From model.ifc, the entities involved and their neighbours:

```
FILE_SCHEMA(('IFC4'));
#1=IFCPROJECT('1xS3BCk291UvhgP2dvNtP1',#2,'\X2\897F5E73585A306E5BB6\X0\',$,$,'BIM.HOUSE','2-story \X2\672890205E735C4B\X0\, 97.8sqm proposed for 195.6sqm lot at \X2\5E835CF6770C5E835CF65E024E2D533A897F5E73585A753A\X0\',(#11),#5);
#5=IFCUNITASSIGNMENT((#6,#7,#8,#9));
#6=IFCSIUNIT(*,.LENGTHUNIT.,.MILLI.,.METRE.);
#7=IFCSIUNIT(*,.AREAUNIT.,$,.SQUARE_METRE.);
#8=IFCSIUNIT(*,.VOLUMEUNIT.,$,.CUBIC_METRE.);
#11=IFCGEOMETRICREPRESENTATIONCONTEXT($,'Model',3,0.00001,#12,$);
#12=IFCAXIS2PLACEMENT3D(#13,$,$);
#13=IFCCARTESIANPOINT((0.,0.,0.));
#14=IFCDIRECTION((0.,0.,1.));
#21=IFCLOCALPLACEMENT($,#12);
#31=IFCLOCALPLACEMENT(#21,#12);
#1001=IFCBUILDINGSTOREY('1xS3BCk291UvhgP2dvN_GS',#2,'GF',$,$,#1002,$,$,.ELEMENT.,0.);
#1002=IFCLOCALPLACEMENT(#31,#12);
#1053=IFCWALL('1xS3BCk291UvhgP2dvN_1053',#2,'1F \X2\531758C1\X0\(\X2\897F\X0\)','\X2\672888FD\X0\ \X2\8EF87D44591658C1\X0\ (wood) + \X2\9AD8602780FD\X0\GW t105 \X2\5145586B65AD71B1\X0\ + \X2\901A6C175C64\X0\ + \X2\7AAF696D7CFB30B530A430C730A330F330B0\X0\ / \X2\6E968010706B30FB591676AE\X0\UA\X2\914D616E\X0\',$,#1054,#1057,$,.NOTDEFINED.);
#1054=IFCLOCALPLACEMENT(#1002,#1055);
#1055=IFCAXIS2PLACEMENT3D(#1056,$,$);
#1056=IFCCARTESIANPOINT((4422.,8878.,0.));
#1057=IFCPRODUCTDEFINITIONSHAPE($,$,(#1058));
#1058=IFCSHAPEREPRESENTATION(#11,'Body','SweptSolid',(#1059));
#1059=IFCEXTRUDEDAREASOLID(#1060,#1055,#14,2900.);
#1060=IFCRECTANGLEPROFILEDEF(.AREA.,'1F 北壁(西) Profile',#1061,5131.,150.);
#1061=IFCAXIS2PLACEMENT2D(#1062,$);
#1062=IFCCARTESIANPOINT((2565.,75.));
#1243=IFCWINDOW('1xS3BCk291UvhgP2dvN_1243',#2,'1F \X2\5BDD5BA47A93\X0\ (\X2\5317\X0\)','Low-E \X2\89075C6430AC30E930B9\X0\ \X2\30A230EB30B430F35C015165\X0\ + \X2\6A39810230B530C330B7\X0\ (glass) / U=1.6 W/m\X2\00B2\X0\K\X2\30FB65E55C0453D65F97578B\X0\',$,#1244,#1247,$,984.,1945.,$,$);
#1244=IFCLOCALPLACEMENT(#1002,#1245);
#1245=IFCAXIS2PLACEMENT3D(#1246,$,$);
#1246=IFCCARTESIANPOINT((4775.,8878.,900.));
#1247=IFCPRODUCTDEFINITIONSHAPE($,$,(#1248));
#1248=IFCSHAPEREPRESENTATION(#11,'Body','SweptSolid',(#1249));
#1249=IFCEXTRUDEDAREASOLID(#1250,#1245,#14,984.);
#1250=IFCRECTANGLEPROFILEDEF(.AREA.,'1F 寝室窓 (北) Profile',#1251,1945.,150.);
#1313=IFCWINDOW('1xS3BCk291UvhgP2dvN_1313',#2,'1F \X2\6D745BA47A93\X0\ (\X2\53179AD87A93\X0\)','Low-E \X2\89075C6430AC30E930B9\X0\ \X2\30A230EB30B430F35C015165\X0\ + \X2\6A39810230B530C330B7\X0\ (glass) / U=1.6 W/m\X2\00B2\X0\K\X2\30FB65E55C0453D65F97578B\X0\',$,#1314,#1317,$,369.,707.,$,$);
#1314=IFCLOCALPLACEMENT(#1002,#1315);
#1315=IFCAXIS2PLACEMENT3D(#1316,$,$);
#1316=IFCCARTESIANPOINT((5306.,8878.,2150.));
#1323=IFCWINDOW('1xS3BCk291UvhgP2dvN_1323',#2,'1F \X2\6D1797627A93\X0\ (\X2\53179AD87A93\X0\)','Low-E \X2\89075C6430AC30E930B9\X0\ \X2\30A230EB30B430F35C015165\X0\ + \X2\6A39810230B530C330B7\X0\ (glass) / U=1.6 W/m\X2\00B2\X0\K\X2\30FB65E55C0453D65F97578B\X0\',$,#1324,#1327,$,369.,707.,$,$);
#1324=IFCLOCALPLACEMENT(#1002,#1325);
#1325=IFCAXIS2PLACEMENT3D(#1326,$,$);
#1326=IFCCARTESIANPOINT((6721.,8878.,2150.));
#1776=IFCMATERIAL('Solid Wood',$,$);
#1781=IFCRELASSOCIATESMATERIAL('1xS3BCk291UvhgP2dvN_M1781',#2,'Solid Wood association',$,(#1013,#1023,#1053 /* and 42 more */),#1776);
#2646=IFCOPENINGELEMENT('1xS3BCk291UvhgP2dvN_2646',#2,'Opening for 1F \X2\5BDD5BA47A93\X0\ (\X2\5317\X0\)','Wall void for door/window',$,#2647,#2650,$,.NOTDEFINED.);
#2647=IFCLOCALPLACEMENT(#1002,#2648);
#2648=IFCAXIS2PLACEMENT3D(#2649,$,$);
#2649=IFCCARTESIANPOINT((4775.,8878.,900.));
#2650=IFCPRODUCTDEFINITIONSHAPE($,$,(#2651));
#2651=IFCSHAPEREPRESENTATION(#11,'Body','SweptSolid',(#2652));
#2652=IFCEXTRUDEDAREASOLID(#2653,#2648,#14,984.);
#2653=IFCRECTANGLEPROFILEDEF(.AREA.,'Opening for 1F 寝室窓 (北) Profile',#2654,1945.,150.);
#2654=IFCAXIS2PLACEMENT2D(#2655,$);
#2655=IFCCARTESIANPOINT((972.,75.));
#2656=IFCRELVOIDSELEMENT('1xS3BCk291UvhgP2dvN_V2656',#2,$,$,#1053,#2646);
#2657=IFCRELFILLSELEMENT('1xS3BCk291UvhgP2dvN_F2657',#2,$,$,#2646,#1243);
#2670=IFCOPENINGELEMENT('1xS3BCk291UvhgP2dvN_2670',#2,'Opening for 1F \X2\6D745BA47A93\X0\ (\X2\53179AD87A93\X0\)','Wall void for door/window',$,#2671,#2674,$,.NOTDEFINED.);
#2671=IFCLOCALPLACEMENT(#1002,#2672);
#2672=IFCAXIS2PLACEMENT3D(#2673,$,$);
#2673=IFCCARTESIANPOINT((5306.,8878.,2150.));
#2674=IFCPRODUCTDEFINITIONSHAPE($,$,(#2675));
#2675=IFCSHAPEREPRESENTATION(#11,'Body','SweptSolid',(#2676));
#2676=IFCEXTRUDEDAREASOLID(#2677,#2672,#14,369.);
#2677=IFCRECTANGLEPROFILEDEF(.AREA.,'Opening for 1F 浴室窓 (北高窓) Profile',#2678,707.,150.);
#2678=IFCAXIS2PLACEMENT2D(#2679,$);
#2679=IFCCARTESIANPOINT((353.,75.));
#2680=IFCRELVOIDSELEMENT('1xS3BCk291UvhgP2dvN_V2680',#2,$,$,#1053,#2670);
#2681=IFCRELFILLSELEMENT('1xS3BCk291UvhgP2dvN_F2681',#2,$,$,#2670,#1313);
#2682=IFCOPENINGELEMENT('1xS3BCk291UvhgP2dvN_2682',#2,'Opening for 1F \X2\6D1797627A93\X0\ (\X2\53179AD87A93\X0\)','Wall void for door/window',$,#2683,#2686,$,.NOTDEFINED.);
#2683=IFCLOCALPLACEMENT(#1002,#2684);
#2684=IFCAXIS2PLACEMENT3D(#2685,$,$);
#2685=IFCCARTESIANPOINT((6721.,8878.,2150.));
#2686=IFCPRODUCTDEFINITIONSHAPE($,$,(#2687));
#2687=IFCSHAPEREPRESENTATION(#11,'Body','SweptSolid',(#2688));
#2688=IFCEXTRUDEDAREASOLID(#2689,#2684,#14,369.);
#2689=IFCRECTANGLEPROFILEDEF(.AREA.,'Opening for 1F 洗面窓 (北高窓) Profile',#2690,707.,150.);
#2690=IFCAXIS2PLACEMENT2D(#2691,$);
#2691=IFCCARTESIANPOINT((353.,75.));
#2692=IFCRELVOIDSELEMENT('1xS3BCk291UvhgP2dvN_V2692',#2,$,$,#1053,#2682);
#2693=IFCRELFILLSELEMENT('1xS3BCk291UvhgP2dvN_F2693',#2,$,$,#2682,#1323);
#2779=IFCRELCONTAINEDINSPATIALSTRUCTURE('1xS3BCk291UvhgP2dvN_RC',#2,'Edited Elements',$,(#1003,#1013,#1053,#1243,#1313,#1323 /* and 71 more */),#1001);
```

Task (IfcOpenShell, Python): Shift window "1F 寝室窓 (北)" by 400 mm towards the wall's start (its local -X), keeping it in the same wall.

```python
import ifcopenshell
import ifcopenshell.api.geometry
import ifcopenshell.util.placement
import ifcopenshell.util.unit

model = ifcopenshell.open("model.ifc")
unit_scale = ifcopenshell.util.unit.calculate_unit_scale(model)

window = model.by_guid("1xS3BCk291UvhgP2dvN_1243")
opening = window.FillsVoids[0].RelatingOpeningElement
wall = opening.VoidsElements[0].RelatingBuildingElement

wall_matrix = ifcopenshell.util.placement.get_local_placement(wall.ObjectPlacement)
shift = wall_matrix[:3, 0] * -0.4 / unit_scale
before = ifcopenshell.util.placement.get_local_placement(window.ObjectPlacement)[:3, 3].copy()

# The window is not placed relative to its opening, so move both.
for product in (opening, window):
    matrix = ifcopenshell.util.placement.get_local_placement(product.ObjectPlacement)
    matrix[:3, 3] += shift
    ifcopenshell.api.geometry.edit_object_placement(model, product=product, matrix=matrix, is_si=False)

after = ifcopenshell.util.placement.get_local_placement(window.ObjectPlacement)[:3, 3]
print("window moved by", (after - before).round(3) + 0.0)

model.write("model_v2.ifc")
```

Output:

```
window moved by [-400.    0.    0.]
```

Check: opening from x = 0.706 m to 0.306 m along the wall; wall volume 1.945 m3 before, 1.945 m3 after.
